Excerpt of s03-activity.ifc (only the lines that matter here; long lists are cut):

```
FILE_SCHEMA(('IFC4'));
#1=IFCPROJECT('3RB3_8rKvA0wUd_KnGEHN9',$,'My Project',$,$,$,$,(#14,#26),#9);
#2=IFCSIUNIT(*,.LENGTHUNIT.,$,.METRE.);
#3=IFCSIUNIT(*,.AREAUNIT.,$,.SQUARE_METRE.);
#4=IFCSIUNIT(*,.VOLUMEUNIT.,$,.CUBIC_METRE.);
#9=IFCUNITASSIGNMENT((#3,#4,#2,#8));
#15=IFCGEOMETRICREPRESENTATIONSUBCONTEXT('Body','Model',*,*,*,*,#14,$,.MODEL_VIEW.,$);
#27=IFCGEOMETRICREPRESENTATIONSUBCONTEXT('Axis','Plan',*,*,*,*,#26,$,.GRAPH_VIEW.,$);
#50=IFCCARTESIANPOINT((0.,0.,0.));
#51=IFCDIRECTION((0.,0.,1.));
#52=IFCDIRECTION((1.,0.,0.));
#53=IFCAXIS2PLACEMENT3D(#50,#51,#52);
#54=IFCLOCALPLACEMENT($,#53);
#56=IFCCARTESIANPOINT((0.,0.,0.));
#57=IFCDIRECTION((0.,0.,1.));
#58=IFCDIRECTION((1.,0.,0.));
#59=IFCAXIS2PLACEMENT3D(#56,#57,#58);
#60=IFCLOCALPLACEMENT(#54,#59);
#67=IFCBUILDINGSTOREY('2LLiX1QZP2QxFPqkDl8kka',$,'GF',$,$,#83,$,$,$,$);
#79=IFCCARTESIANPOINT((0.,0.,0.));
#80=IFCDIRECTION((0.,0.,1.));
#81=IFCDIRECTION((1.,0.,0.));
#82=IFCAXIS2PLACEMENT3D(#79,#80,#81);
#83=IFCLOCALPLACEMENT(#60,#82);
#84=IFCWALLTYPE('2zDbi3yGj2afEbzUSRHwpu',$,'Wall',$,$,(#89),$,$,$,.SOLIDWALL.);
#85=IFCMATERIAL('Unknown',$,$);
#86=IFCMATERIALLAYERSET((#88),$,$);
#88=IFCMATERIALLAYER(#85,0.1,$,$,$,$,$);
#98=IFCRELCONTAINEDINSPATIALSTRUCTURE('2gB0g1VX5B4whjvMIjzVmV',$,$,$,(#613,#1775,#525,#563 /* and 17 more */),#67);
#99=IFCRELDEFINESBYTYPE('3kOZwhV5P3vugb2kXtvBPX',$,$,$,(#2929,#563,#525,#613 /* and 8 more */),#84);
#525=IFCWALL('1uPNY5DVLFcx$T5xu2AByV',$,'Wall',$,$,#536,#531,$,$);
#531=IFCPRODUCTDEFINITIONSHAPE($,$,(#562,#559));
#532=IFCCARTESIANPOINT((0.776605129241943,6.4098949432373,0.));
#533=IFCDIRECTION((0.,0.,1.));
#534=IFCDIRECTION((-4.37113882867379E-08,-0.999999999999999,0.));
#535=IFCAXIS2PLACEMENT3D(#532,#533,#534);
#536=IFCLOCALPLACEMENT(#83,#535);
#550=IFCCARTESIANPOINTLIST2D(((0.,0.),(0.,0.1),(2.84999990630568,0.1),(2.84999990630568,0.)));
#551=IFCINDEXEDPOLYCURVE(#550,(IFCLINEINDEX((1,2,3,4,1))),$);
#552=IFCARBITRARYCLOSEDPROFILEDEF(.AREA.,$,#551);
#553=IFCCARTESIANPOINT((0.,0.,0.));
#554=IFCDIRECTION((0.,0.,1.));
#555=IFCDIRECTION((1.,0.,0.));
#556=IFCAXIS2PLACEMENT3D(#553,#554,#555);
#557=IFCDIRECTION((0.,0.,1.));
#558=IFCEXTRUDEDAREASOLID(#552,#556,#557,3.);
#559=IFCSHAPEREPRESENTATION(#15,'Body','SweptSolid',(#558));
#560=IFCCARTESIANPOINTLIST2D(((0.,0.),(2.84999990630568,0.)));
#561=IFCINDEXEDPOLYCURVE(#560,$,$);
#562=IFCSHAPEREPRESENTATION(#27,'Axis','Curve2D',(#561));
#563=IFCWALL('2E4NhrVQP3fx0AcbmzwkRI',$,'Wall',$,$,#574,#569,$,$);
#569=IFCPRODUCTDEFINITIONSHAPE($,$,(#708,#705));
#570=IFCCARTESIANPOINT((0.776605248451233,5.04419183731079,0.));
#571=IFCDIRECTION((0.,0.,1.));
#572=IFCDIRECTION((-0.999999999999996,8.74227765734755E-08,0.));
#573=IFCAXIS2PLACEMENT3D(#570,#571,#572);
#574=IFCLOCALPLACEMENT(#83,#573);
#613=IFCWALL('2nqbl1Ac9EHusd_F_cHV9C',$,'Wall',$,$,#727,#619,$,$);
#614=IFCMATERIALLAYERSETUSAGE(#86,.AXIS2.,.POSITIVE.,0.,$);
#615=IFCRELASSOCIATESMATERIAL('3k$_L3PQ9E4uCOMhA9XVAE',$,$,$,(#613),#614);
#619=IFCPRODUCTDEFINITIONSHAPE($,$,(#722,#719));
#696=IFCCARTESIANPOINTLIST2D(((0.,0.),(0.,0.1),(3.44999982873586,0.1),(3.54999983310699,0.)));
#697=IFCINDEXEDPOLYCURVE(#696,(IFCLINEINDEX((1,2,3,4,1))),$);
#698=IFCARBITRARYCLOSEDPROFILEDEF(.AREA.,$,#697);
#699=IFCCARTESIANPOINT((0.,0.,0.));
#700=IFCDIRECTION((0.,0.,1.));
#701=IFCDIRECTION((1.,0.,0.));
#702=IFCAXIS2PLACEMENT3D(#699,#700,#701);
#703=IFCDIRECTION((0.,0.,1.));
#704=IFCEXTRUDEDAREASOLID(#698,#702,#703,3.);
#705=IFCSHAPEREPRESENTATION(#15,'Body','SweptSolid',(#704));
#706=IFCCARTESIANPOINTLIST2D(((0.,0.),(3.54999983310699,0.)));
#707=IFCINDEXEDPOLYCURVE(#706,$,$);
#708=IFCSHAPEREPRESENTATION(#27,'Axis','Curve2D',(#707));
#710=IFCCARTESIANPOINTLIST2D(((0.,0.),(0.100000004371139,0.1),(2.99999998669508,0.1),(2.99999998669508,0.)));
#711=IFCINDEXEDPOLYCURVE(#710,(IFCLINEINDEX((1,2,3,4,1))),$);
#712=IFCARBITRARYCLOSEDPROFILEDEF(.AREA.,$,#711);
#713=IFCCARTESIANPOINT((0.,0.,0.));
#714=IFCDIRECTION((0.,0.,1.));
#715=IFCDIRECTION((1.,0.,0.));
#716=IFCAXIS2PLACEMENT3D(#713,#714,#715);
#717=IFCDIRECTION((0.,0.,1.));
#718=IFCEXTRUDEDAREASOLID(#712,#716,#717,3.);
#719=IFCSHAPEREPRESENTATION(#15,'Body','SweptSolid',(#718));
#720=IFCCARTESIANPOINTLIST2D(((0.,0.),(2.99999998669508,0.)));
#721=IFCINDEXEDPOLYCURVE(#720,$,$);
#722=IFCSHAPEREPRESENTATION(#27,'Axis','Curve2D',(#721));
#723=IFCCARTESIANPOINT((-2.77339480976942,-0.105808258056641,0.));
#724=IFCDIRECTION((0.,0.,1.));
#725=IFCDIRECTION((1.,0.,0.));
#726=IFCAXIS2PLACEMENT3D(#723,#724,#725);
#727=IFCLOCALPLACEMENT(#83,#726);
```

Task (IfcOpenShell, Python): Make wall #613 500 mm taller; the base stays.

```python
import ifcopenshell
import ifcopenshell.geom
import ifcopenshell.util.representation
import ifcopenshell.util.shape
import ifcopenshell.util.unit

model = ifcopenshell.open("s03-activity.ifc")
unit_scale = ifcopenshell.util.unit.calculate_unit_scale(model)
settings = ifcopenshell.geom.settings()


def volume(element):
    """Net volume in cubic metres, openings subtracted."""
    shape = ifcopenshell.geom.create_shape(settings, element)
    return ifcopenshell.util.shape.get_volume(shape.geometry)


wall = model.by_id(613)
before = volume(wall)

body = ifcopenshell.util.representation.get_representation(wall, "Model", "Body")
solid = body.Items[0]
old_height = solid.Depth
solid.Depth += 0.5 / unit_scale
after = volume(wall)

print(f"height {old_height:g} -> {solid.Depth:g}, volume {before:.3f} -> {after:.3f} m3")

model.write("s03-activity_v2.ifc")
```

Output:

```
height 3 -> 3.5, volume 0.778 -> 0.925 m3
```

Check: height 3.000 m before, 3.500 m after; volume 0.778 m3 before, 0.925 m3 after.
